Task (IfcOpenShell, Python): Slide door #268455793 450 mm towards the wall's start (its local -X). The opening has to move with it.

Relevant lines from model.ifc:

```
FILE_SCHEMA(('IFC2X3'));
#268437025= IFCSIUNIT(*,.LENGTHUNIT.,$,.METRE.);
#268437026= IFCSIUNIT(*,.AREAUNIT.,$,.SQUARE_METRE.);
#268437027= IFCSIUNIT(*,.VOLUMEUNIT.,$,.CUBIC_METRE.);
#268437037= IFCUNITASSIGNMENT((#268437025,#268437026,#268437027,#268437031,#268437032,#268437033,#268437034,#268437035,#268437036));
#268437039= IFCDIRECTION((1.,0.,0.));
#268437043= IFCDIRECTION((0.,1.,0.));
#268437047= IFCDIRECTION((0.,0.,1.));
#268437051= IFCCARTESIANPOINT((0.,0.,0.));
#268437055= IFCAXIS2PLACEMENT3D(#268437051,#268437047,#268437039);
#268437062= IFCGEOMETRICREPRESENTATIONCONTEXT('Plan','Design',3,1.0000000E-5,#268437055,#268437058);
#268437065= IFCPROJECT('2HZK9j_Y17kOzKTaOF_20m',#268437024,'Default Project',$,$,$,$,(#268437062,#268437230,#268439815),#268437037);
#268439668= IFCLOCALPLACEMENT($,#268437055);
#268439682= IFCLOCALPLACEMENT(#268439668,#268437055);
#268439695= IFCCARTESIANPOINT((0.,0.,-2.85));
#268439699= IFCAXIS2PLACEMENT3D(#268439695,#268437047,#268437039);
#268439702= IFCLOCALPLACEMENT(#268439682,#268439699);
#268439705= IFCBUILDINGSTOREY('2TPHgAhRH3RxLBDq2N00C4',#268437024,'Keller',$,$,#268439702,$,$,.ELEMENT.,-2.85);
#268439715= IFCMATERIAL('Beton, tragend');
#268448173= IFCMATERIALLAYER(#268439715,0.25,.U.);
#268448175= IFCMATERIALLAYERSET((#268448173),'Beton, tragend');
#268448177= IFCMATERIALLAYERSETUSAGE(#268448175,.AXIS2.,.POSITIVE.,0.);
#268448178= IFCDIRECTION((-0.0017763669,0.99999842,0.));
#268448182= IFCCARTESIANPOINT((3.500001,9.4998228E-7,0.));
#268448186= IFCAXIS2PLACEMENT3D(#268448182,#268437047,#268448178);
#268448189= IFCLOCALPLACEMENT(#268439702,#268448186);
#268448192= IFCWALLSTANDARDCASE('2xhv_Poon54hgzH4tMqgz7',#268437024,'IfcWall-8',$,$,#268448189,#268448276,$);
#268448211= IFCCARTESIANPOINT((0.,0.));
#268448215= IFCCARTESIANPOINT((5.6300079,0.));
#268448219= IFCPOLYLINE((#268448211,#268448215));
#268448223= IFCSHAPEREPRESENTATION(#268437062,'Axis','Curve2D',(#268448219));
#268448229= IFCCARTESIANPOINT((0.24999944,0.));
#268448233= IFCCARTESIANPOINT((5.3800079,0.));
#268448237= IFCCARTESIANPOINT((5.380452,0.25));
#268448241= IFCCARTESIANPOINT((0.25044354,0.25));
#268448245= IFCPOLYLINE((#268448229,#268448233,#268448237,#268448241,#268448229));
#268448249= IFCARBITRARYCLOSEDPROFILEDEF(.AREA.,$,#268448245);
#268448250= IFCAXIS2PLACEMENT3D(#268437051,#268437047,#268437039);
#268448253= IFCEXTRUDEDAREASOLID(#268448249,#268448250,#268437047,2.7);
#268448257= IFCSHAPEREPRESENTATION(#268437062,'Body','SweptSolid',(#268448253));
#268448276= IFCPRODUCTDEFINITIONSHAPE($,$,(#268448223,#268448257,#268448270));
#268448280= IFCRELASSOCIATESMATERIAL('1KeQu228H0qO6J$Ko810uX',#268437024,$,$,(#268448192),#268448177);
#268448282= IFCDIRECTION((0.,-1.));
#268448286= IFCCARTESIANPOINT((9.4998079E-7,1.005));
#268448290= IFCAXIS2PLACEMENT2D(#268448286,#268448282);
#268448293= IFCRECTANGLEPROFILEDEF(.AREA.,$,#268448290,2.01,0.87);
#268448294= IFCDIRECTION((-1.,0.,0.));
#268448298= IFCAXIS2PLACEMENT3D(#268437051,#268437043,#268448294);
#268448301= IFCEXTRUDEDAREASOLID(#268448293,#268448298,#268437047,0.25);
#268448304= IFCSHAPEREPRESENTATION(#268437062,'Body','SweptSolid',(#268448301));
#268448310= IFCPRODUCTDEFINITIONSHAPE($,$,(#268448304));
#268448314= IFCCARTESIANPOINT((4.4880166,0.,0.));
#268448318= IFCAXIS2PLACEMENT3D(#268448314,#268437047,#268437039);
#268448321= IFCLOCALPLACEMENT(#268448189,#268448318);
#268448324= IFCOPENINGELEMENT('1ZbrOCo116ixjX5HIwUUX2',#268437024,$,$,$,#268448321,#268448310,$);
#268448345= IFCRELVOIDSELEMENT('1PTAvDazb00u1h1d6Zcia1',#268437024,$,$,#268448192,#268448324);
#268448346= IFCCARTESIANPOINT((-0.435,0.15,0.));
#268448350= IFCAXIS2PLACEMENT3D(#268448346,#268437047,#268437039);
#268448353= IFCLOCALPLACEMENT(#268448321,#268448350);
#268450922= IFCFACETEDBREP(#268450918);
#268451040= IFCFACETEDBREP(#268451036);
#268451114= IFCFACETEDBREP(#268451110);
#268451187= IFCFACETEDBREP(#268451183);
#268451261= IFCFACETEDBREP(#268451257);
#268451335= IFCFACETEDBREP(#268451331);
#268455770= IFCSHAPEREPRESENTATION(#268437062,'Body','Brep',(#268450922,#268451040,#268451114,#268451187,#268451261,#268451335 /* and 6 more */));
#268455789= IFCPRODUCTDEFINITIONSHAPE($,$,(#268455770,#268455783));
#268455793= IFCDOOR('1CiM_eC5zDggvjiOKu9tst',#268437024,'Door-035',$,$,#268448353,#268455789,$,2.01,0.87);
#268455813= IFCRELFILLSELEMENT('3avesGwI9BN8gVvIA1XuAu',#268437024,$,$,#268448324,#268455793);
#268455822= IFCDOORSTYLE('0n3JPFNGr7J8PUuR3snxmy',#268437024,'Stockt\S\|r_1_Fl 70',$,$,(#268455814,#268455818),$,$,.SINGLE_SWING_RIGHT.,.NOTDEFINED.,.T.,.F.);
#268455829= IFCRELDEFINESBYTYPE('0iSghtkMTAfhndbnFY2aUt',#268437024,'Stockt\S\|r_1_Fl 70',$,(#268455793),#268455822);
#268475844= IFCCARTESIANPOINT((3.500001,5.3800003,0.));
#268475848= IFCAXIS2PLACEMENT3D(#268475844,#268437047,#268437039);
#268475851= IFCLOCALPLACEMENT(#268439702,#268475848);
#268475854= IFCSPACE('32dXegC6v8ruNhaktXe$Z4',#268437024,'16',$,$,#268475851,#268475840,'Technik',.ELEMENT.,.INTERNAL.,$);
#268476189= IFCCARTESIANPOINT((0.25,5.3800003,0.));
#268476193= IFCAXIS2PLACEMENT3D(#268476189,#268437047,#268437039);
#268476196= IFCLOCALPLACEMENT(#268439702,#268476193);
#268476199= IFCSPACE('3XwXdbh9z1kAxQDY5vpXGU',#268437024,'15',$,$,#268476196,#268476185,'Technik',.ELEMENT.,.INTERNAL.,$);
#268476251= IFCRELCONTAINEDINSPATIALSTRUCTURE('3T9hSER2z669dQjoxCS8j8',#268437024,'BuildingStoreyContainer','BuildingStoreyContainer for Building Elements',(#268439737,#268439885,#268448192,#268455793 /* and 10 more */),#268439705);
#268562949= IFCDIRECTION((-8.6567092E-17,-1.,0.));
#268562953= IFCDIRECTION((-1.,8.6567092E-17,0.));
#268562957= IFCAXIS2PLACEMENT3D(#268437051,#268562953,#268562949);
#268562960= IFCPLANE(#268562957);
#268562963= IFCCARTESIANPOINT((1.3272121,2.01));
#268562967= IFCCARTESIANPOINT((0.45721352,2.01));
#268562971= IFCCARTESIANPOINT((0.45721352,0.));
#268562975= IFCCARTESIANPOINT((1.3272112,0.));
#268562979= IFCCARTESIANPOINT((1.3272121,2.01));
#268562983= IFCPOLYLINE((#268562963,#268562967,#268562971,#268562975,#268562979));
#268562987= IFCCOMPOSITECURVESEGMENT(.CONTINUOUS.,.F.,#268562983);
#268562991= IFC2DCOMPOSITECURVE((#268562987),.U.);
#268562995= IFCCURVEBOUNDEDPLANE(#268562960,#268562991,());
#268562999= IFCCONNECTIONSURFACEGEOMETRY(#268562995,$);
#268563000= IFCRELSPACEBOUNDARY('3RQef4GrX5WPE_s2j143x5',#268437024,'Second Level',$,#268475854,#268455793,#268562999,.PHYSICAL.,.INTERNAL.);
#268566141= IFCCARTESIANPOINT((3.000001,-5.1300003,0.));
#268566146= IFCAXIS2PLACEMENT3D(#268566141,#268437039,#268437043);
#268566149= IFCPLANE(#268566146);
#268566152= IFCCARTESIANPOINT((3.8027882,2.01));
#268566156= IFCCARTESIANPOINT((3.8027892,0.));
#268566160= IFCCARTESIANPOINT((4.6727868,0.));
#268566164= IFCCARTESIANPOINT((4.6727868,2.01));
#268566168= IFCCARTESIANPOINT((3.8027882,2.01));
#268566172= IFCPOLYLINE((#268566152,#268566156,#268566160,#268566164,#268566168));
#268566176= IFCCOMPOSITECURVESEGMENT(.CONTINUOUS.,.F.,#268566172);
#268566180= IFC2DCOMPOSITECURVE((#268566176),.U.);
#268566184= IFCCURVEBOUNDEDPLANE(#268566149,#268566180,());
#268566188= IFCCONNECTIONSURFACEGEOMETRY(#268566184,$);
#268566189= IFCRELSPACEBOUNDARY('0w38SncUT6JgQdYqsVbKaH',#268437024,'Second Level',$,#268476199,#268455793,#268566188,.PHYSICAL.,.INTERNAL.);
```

```python
import numpy as np
import ifcopenshell
import ifcopenshell.api.geometry
import ifcopenshell.util.placement

model = ifcopenshell.open("model.ifc")

door = model.by_guid("1CiM_eC5zDggvjiOKu9tst")
opening = door.FillsVoids[0].RelatingOpeningElement
wall = opening.VoidsElements[0].RelatingBuildingElement

wall_matrix = ifcopenshell.util.placement.get_local_placement(wall.ObjectPlacement)
shift = wall_matrix[:3, 0] * -0.45
before = ifcopenshell.util.placement.get_local_placement(door.ObjectPlacement)[:3, 3].copy()

# The door is placed relative to its opening, so it follows when the opening moves.
matrix = ifcopenshell.util.placement.get_local_placement(opening.ObjectPlacement)
matrix[:3, 3] += shift
ifcopenshell.api.geometry.edit_object_placement(
    model, product=opening, matrix=matrix, is_si=False, should_transform_children=True
)

# Space boundary surfaces are stored in each space's coordinates; move them too.
for rel in door.ProvidesBoundaries:
    if not rel.ConnectionGeometry:
        continue
    surface = rel.ConnectionGeometry.SurfaceOnRelatingElement.BasisSurface
    space_matrix = ifcopenshell.util.placement.get_local_placement(rel.RelatingSpace.ObjectPlacement)
    point = np.array(surface.Position.Location.Coordinates) + space_matrix[:3, :3].T @ shift
    surface.Position = model.createIfcAxis2Placement3D(
        model.createIfcCartesianPoint(point.tolist()), surface.Position.Axis, surface.Position.RefDirection
    )

after = ifcopenshell.util.placement.get_local_placement(door.ObjectPlacement)[:3, 3]
print("door moved by", (after - before).round(3) + 0.0)

model.write("model_edited.ifc")
```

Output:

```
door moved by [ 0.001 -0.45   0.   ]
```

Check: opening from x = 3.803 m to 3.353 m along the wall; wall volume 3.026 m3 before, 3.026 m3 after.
